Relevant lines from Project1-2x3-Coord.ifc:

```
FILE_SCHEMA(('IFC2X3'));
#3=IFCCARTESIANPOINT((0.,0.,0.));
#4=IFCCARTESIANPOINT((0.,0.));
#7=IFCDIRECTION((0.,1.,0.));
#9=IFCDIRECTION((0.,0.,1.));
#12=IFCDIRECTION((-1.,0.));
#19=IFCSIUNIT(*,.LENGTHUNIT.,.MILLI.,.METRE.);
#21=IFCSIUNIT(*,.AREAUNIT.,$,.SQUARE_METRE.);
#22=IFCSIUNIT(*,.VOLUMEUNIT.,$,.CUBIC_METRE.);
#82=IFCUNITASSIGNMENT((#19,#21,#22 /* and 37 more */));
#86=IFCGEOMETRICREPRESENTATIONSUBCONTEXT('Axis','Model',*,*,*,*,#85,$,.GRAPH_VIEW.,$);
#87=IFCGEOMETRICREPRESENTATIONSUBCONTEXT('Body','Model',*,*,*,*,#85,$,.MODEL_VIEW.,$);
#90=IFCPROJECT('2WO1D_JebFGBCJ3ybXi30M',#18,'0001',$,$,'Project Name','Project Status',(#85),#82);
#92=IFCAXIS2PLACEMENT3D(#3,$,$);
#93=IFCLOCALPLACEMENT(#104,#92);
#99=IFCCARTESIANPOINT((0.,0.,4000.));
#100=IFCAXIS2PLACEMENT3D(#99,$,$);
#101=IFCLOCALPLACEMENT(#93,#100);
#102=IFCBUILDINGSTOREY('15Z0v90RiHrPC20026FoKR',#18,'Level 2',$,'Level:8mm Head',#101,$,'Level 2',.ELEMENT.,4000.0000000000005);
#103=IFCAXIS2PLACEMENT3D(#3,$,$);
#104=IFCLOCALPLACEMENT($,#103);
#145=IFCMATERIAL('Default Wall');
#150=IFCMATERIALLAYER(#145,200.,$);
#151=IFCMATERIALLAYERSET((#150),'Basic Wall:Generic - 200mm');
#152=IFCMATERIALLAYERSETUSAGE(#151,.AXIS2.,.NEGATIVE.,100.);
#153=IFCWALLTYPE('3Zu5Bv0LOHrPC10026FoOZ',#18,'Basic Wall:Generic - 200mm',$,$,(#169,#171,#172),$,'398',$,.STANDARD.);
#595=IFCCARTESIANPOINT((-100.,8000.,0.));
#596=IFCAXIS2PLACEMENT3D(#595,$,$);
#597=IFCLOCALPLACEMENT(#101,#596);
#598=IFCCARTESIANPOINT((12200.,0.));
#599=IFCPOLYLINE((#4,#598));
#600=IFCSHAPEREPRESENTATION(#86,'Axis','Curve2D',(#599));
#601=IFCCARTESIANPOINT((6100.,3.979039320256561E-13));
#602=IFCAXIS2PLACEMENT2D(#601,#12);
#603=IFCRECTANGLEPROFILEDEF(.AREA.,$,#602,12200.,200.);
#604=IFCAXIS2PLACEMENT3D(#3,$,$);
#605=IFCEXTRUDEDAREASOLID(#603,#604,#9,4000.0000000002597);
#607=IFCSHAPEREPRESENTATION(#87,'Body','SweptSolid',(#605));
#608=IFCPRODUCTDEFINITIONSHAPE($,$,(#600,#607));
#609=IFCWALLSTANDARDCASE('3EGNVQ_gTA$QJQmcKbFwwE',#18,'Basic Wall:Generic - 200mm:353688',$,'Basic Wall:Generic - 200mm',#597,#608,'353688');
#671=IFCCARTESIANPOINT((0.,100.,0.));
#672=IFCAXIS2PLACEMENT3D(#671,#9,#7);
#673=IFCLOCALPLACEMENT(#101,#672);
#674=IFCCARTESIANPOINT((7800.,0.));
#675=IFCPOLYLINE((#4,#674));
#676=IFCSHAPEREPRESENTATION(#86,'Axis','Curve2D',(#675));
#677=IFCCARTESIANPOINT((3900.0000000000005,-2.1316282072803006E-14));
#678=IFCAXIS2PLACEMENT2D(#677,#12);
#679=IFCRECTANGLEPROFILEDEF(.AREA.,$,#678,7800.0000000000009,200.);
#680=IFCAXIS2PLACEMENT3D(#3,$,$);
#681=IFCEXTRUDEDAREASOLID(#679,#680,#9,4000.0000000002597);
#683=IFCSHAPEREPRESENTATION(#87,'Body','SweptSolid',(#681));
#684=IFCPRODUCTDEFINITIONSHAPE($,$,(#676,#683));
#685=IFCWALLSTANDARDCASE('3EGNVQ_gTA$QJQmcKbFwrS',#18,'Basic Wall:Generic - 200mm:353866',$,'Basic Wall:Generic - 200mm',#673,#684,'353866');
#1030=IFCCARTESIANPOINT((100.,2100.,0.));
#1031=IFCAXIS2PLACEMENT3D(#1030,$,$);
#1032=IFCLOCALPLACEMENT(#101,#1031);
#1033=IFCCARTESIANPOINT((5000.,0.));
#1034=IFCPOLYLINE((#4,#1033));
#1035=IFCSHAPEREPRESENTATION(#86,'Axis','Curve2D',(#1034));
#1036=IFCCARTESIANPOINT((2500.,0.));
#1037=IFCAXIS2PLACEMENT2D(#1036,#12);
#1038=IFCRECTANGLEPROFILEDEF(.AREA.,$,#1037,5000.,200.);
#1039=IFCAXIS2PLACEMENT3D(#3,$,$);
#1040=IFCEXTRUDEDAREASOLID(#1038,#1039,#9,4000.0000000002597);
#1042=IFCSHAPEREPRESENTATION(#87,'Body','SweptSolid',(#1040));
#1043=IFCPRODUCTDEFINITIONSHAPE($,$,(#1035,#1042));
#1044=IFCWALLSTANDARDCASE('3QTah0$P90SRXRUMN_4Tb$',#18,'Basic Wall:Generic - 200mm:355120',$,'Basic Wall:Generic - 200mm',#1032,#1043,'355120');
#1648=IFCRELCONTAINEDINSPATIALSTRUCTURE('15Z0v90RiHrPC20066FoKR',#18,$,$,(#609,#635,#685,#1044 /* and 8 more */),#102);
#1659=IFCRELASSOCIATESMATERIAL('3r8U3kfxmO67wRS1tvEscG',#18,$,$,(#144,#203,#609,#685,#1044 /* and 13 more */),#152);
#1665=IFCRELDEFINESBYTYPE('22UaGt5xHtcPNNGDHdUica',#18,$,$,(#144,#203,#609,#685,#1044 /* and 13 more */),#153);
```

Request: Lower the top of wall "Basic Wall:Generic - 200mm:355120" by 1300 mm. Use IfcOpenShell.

```python
import ifcopenshell
import ifcopenshell.geom
import ifcopenshell.util.representation
import ifcopenshell.util.shape

model = ifcopenshell.open("Project1-2x3-Coord.ifc")
settings = ifcopenshell.geom.settings()


def volume(element):
    """Net volume in cubic metres, openings subtracted."""
    shape = ifcopenshell.geom.create_shape(settings, element)
    return ifcopenshell.util.shape.get_volume(shape.geometry)


wall = model.by_id(1044)
before = volume(wall)

body = ifcopenshell.util.representation.get_representation(wall, "Model", "Body")
solid = body.Items[0]
old_height = solid.Depth
solid.Depth -= 1300.0
after = volume(wall)

print(f"height {old_height:g} -> {solid.Depth:g}, volume {before:.3f} -> {after:.3f} m3")

model.write("Project1-2x3-Coord-out.ifc")
```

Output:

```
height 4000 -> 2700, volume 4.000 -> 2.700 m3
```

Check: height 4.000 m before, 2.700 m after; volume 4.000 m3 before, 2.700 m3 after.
